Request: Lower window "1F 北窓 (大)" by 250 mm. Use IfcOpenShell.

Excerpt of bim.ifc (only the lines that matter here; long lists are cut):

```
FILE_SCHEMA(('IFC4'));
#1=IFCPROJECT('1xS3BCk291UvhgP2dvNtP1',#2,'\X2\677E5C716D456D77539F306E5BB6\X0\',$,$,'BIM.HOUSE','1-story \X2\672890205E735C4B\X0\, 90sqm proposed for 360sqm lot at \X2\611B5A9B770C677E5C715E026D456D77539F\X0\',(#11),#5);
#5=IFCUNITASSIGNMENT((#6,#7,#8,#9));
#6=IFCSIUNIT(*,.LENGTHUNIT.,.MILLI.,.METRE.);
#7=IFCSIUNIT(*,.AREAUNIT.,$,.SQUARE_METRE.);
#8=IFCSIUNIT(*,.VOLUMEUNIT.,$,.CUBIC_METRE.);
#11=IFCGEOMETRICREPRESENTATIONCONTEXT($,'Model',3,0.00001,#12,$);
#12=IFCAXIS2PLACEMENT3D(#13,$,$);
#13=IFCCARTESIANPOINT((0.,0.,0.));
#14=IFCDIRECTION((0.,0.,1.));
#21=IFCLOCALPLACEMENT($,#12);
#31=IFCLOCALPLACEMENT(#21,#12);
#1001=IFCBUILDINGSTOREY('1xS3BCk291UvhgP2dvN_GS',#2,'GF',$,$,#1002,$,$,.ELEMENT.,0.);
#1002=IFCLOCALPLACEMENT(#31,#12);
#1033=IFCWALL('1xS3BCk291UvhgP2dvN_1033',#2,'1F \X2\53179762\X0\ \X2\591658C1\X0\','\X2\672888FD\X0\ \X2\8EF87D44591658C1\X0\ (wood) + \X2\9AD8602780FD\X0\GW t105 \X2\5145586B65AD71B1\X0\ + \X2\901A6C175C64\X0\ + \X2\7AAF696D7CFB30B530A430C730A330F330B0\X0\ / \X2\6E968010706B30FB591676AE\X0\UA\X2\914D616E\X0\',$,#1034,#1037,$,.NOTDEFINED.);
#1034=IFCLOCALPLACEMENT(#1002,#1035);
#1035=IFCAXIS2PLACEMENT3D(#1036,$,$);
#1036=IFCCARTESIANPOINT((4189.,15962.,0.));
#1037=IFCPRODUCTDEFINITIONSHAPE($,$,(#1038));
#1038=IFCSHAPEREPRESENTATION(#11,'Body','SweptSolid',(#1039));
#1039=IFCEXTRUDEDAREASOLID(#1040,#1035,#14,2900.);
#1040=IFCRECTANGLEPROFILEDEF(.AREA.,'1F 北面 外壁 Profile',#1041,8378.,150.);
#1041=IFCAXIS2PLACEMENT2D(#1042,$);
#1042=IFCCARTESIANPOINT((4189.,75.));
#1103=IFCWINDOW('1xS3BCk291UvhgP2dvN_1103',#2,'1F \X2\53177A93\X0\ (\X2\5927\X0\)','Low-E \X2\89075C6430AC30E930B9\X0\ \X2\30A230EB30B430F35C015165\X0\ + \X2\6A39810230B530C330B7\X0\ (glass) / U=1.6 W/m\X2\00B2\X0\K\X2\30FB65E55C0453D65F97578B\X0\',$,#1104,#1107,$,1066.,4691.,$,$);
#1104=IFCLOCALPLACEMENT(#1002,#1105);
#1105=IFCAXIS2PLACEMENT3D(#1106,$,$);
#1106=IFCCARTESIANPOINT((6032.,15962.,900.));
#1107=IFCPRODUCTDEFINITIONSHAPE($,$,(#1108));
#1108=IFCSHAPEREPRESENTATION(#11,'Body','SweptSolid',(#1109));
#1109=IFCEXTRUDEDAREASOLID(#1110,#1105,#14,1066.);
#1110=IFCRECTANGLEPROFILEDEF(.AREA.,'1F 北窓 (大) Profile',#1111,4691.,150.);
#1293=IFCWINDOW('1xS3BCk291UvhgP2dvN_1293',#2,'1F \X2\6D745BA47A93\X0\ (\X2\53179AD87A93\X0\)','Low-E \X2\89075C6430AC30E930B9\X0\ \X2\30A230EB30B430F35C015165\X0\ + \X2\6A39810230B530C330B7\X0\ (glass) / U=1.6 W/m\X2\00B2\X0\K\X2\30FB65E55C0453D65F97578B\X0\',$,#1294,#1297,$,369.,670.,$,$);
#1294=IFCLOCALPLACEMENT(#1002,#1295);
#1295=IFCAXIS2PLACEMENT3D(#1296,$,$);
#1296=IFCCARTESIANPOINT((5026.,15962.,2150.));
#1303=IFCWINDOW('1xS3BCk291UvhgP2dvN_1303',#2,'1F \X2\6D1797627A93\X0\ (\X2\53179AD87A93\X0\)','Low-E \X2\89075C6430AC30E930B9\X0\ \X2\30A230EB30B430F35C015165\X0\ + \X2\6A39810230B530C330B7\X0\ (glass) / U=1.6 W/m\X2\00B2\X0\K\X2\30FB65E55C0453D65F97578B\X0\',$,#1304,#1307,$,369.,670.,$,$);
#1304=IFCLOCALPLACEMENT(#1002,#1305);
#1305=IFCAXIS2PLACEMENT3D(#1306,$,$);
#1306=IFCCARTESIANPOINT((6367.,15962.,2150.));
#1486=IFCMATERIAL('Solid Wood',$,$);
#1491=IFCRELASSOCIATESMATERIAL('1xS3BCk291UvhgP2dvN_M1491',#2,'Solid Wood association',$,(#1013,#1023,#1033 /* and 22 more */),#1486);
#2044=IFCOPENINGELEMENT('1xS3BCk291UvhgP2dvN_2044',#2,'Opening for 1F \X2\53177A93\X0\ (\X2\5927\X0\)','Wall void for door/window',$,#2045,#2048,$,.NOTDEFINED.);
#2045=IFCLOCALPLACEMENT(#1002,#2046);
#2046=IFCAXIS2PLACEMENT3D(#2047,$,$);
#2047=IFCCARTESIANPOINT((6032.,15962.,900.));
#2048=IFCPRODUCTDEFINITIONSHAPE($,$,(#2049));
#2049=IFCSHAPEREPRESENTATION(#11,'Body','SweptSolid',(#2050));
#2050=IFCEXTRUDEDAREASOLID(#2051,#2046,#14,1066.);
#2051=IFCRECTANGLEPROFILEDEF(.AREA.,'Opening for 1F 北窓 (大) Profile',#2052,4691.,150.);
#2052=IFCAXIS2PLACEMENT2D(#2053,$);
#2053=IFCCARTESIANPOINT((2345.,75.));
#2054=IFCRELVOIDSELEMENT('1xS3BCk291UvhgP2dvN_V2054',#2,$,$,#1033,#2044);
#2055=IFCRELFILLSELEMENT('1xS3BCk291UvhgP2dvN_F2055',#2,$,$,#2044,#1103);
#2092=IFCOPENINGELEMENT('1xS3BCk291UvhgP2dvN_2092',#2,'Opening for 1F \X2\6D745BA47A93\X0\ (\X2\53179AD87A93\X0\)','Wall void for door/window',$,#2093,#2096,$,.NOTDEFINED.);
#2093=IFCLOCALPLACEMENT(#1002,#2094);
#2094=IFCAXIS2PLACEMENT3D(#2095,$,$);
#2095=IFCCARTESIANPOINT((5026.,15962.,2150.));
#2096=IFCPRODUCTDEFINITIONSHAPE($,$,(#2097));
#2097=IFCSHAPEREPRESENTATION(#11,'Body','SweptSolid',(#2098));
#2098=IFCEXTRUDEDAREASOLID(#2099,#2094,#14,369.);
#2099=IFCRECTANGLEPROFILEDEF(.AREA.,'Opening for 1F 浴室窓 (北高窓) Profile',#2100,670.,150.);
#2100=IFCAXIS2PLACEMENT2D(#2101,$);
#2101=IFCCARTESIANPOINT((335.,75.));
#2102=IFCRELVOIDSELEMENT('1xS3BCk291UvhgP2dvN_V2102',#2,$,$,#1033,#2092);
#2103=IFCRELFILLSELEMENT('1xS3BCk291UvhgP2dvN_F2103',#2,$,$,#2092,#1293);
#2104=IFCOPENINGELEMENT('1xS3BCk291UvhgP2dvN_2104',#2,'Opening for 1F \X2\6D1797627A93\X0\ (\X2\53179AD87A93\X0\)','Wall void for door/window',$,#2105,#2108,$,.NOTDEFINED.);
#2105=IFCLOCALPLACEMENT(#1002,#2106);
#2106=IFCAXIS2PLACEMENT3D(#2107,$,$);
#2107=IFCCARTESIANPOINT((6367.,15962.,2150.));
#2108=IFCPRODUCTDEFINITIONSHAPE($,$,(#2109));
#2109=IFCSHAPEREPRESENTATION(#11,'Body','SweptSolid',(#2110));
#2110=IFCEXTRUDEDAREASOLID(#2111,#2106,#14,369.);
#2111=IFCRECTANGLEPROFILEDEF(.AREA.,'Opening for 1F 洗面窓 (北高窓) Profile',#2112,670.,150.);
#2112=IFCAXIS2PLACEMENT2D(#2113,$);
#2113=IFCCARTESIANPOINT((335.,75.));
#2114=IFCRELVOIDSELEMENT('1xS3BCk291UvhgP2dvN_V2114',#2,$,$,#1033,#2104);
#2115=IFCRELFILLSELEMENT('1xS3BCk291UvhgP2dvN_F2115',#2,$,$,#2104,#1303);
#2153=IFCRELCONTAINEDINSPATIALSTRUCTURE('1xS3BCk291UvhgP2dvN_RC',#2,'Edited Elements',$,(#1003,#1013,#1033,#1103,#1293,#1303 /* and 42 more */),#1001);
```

```python
import numpy as np
import ifcopenshell
import ifcopenshell.api.geometry
import ifcopenshell.util.placement
import ifcopenshell.util.unit

model = ifcopenshell.open("bim.ifc")
unit_scale = ifcopenshell.util.unit.calculate_unit_scale(model)

window = model.by_guid("1xS3BCk291UvhgP2dvN_1103")
opening = window.FillsVoids[0].RelatingOpeningElement
dz = -250.0

shift = np.array([0.0, 0.0, dz])
# The window is not placed relative to its opening, so move both.
for product in (opening, window):
    matrix = ifcopenshell.util.placement.get_local_placement(product.ObjectPlacement)
    matrix[:3, 3] += shift
    ifcopenshell.api.geometry.edit_object_placement(model, product=product, matrix=matrix, is_si=False)

print(f"moved by {dz * unit_scale:+.3f} m")

model.write("bim_v2.ifc")
```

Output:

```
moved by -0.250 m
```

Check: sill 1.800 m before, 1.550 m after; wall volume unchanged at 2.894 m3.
